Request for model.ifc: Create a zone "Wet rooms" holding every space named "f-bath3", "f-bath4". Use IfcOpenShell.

First a look at what the model holds.

```python
import ifcopenshell

model = ifcopenshell.open("model.ifc")
print(model.schema)
seen = {}
for space in model.by_type("IfcSpace"):
    seen[space.LongName] = seen.get(space.LongName, 0) + 1
for name, count in sorted(seen.items(), key=str):
    print(count, "x", name)
print("zones:", [z.Name for z in model.by_type("IfcZone")][:20])
```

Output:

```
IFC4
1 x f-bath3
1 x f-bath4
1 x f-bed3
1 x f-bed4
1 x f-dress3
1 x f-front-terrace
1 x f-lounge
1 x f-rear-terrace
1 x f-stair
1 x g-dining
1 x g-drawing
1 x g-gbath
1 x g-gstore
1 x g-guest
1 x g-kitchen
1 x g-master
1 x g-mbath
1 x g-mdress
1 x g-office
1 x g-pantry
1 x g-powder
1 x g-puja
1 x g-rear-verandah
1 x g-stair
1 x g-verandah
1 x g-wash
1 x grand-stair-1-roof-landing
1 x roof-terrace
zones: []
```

```python
import ifcopenshell
import ifcopenshell.api.group
import ifcopenshell.api.root

model = ifcopenshell.open("model.ifc")

names = {"f-bath3", "f-bath4"}
spaces = [s for s in model.by_type("IfcSpace") if s.LongName in names]

zone = ifcopenshell.api.root.create_entity(model, ifc_class="IfcZone", name="Wet rooms")
ifcopenshell.api.group.assign_group(model, products=spaces, group=zone)
print(len(spaces), "spaces in", zone.Name)

model.write("model_rev.ifc")
```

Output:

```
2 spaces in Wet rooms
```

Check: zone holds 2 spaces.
